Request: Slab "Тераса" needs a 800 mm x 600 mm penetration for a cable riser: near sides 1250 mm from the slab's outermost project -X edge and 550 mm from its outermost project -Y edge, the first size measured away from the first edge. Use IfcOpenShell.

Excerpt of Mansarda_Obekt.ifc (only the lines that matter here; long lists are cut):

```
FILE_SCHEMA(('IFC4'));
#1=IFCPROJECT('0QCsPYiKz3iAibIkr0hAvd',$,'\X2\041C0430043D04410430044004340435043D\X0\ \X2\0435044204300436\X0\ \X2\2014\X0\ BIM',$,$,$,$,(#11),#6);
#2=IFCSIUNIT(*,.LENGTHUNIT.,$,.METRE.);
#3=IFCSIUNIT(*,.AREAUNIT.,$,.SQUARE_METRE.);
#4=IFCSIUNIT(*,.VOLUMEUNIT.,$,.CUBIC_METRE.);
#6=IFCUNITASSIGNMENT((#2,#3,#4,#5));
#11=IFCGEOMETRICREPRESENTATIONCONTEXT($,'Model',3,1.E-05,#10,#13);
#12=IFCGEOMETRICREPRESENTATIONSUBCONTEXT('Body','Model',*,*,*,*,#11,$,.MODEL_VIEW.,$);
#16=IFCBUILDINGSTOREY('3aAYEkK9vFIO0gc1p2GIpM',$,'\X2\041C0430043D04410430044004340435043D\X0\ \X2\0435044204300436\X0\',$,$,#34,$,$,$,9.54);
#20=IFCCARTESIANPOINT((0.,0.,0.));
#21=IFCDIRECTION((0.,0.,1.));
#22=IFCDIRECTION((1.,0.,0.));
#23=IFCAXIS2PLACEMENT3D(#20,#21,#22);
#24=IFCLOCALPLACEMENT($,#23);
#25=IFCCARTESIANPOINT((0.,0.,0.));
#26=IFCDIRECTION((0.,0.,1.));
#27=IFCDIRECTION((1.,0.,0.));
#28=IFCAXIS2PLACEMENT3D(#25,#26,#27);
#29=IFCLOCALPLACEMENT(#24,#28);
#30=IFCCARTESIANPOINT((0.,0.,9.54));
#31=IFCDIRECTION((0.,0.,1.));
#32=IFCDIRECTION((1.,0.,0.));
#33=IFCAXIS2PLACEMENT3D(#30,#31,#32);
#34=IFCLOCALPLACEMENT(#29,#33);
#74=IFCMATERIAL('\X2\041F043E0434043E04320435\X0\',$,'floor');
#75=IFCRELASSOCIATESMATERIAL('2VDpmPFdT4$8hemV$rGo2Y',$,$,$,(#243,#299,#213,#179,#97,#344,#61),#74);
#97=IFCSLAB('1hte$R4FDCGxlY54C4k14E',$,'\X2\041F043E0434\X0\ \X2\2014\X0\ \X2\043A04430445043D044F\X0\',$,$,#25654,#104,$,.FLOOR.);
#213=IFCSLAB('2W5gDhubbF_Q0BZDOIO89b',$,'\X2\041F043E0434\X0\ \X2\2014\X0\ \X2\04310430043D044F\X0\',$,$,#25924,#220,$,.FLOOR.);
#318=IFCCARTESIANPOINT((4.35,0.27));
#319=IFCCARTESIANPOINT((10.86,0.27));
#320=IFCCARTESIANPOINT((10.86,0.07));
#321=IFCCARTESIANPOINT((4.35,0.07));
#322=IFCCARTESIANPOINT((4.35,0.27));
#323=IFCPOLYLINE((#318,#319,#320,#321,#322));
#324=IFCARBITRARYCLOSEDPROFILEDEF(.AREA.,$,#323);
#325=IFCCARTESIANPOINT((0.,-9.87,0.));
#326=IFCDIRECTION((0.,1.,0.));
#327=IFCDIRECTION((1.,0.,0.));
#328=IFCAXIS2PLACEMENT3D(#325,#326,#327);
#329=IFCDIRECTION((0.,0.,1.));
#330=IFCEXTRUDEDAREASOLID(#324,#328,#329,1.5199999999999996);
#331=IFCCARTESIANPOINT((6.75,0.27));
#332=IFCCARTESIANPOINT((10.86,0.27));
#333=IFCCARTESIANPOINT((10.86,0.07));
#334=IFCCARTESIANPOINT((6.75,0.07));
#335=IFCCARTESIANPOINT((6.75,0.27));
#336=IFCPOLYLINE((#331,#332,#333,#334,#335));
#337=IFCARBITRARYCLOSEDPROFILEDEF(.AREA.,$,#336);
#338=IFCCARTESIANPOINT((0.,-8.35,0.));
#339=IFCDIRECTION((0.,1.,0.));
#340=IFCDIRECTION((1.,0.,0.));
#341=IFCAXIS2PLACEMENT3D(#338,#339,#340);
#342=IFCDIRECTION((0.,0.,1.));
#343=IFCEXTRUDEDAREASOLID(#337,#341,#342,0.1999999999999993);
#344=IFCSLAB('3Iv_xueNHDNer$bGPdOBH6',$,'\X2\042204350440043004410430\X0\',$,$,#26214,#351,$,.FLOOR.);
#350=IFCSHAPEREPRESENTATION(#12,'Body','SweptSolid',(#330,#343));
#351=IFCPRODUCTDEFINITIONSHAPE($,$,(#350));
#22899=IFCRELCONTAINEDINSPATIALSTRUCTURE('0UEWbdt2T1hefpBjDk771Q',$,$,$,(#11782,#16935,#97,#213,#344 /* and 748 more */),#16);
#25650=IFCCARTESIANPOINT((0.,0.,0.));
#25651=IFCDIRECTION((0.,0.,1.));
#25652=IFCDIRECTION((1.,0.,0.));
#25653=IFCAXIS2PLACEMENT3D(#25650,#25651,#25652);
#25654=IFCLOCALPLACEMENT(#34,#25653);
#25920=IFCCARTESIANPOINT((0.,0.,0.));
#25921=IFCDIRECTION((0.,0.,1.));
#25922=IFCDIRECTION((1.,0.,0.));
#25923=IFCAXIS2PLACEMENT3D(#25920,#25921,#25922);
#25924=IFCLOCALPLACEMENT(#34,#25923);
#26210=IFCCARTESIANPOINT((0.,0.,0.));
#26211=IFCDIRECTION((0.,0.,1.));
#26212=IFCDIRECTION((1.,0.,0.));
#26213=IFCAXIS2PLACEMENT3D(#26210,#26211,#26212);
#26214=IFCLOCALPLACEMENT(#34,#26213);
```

```python
import numpy as np
import ifcopenshell
import ifcopenshell.api.feature
import ifcopenshell.api.geometry
import ifcopenshell.api.root
import ifcopenshell.geom
import ifcopenshell.util.placement
import ifcopenshell.util.representation
import ifcopenshell.util.shape
import ifcopenshell.util.unit

model = ifcopenshell.open("Mansarda_Obekt.ifc")
unit_scale = ifcopenshell.util.unit.calculate_unit_scale(model)
settings = ifcopenshell.geom.settings()


def volume(element):
    """Net volume in cubic metres, openings subtracted."""
    shape = ifcopenshell.geom.create_shape(settings, element)
    return ifcopenshell.util.shape.get_volume(shape.geometry)


slab = model.by_guid("3Iv_xueNHDNer$bGPdOBH6")
before = volume(slab)

# Extent in the slab's own axes, in metres. The edges named are its -X and -Y sides.
slab_shape = ifcopenshell.geom.create_shape(settings, slab)
vertices = ifcopenshell.util.shape.get_vertices(slab_shape.geometry)
x_min, y_min, bottom = vertices.min(axis=0)
top = vertices[:, 2].max()

opening = ifcopenshell.api.root.create_entity(model, ifc_class="IfcOpeningElement", name="Cable riser opening", predefined_type="OPENING")
context = ifcopenshell.util.representation.get_context(model, "Model", "Body", "MODEL_VIEW")
width, depth = 0.8, 0.6
outline = [(0.0, 0.0), (width, 0.0), (width, depth), (0.0, depth), (0.0, 0.0)]
# Overshoot both faces by 50 mm so the cut is clean.
shape = ifcopenshell.api.geometry.add_slab_representation(
    model, context=context, depth=top - bottom + 0.1, polyline=outline
)
ifcopenshell.api.geometry.assign_representation(model, product=opening, representation=shape)

matrix = ifcopenshell.util.placement.get_local_placement(slab.ObjectPlacement)
matrix[:, 3] = matrix @ np.append(np.array([x_min + 1.25, y_min + 0.55, bottom - 0.05]) / unit_scale, 1.0)
ifcopenshell.api.geometry.edit_object_placement(model, product=opening, matrix=matrix, is_si=False)
ifcopenshell.api.feature.add_feature(model, feature=opening, element=slab)

after = volume(slab)

print(f"slab volume {before:.3f} -> {after:.3f} m3")

model.write("Mansarda_Obekt_rev.ifc")
```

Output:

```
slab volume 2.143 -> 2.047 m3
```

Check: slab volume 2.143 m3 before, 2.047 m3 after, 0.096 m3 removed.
